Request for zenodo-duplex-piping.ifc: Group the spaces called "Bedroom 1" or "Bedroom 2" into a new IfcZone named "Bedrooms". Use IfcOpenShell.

First a look at what the model holds.

```python
import ifcopenshell

model = ifcopenshell.open("zenodo-duplex-piping.ifc")
print(model.schema)
seen = {}
for space in model.by_type("IfcSpace"):
    seen[space.LongName] = seen.get(space.LongName, 0) + 1
for name, count in sorted(seen.items(), key=str):
    print(count, "x", name)
print("zones:", [z.Name for z in model.by_type("IfcZone")][:20])
```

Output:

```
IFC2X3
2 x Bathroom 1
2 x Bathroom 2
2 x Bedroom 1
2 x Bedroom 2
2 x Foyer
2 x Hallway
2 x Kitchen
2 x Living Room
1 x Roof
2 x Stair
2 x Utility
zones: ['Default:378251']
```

```python
import ifcopenshell
import ifcopenshell.api.group
import ifcopenshell.api.root

model = ifcopenshell.open("zenodo-duplex-piping.ifc")

names = {"Bedroom 1", "Bedroom 2"}
spaces = [s for s in model.by_type("IfcSpace") if s.LongName in names]

zone = ifcopenshell.api.root.create_entity(model, ifc_class="IfcZone", name="Bedrooms")
ifcopenshell.api.group.assign_group(model, products=spaces, group=zone)
print(len(spaces), "spaces in", zone.Name)

model.write("zenodo-duplex-piping-out.ifc")
```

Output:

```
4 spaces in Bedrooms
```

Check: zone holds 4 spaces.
